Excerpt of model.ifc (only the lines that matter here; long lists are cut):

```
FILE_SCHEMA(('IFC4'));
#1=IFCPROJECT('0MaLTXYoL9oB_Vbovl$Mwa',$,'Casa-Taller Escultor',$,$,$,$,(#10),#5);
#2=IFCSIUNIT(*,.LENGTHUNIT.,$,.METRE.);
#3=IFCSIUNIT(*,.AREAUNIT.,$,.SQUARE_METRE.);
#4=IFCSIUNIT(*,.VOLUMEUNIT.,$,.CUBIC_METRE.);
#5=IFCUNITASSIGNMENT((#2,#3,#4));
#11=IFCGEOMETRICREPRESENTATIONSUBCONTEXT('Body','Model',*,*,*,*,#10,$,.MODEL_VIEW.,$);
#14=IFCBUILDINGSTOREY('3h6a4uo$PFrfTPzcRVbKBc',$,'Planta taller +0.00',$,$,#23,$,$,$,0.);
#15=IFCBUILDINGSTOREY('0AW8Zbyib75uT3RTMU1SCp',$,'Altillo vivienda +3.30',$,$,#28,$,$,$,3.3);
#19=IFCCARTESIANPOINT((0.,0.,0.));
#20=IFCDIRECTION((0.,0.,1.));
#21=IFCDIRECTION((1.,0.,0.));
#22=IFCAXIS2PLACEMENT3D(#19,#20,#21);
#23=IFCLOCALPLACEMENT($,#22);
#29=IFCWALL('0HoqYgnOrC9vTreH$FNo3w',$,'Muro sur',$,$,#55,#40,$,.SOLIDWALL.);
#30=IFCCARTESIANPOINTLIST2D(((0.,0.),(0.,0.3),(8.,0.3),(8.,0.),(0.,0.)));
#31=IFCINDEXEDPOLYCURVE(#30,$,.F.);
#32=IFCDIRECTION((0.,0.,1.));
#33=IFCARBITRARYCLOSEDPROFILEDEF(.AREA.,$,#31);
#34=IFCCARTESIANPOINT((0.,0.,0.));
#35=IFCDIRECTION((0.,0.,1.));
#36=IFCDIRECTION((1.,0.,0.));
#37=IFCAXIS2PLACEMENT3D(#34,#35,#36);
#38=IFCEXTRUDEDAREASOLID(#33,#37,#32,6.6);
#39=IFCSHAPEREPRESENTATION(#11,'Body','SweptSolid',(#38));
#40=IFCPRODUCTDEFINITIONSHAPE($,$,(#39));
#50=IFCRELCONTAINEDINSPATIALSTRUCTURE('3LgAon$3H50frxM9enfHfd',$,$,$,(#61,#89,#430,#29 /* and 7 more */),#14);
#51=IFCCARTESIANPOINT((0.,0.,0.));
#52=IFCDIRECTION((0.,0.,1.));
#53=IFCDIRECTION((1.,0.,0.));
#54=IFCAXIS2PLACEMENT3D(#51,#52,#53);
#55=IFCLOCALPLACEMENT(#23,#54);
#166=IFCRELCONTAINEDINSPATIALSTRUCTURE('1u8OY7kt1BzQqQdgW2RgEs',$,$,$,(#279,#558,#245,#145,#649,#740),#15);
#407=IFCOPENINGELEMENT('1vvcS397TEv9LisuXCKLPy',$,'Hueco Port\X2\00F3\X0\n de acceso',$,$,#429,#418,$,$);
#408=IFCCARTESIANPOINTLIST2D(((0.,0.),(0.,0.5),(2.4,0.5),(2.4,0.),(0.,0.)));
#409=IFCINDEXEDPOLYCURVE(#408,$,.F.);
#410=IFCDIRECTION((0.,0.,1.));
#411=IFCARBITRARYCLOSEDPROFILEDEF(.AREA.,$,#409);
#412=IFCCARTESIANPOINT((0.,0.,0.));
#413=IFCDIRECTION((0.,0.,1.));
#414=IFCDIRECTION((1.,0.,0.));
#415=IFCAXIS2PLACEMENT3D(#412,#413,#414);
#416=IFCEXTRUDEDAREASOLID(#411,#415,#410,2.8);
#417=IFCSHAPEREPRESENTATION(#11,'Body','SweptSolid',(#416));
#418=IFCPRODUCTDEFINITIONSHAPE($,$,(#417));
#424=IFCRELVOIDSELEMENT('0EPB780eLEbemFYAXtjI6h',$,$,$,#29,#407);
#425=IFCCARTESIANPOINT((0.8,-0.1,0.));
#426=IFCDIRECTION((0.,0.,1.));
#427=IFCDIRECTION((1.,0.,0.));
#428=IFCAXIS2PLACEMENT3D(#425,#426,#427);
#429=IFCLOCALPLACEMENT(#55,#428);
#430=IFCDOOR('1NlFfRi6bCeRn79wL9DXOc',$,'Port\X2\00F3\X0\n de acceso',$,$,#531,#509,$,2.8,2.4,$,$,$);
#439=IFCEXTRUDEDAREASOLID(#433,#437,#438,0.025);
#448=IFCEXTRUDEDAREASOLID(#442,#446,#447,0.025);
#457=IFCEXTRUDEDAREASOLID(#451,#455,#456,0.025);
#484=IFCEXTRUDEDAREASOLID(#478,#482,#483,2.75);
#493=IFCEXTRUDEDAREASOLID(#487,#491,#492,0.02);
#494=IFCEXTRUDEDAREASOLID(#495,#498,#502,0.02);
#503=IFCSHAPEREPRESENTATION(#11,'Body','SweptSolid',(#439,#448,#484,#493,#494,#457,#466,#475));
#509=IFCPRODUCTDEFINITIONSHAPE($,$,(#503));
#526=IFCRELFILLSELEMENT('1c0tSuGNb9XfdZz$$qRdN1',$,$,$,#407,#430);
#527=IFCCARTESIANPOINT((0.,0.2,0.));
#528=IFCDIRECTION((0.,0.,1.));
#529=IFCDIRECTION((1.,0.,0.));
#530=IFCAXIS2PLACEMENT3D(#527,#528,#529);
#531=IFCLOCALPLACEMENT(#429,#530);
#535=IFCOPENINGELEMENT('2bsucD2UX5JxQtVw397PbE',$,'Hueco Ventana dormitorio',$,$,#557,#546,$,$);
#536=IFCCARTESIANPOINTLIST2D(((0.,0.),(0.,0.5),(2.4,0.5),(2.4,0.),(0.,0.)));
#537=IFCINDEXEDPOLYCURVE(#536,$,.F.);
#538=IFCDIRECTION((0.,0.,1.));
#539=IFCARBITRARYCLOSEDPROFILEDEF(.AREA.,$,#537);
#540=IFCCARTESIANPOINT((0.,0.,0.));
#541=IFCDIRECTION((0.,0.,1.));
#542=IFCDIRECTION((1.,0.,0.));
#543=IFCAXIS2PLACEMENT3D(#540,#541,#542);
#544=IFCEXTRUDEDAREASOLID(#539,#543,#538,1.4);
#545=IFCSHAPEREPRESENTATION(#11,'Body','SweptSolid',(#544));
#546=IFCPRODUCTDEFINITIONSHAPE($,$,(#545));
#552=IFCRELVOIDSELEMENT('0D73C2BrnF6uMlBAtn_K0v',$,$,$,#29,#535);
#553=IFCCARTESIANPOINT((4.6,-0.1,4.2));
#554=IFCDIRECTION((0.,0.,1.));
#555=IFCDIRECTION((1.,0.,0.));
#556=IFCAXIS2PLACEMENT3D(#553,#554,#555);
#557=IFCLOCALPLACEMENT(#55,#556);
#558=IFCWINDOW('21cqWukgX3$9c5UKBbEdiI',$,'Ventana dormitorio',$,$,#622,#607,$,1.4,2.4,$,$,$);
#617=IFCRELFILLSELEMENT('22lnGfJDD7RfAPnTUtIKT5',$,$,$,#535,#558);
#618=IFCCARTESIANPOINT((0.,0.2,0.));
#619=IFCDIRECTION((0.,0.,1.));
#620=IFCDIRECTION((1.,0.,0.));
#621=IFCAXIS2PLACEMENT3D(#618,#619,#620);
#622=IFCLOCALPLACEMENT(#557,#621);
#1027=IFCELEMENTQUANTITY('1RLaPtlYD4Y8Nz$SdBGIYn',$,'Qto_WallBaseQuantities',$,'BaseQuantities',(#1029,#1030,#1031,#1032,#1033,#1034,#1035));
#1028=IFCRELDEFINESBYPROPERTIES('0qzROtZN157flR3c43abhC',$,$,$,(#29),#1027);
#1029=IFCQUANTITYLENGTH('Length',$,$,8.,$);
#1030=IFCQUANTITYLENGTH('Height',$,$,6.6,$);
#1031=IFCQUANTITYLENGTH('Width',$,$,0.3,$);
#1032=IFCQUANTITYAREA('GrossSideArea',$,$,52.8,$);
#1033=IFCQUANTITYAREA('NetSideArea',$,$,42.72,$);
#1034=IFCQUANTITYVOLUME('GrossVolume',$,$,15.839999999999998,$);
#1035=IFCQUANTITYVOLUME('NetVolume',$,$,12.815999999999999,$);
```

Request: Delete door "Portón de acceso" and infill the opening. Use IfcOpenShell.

```python
import ifcopenshell
import ifcopenshell.api.feature
import ifcopenshell.api.pset
import ifcopenshell.api.root
import ifcopenshell.geom
import ifcopenshell.util.element
import ifcopenshell.util.shape
import ifcopenshell.util.unit

model = ifcopenshell.open("model.ifc")
area_scale = ifcopenshell.util.unit.calculate_unit_scale(model, "AREAUNIT")
volume_scale = ifcopenshell.util.unit.calculate_unit_scale(model, "VOLUMEUNIT")
settings = ifcopenshell.geom.settings()


def volume(element):
    """Net volume in cubic metres, openings subtracted."""
    shape = ifcopenshell.geom.create_shape(settings, element)
    return ifcopenshell.util.shape.get_volume(shape.geometry)


door = model.by_id(430)
opening = door.FillsVoids[0].RelatingOpeningElement
wall = opening.VoidsElements[0].RelatingBuildingElement
before = volume(wall)

ifcopenshell.api.root.remove_product(model, product=door)
ifcopenshell.api.feature.remove_feature(model, feature=opening)

after = volume(wall)
thickness = 0.3  # wall thickness in metres

# Update the wall's stored quantities.
qto = model.by_id(ifcopenshell.util.element.get_pset(wall, "Qto_WallBaseQuantities", should_inherit=False)["id"])
ifcopenshell.api.pset.edit_qto(model, qto=qto, properties={
    "NetSideArea": after / thickness / area_scale,
    "NetVolume": after / volume_scale,
})

print(f"wall volume {before:.3f} -> {after:.3f} m3")

model.write("model_edited.ifc")
```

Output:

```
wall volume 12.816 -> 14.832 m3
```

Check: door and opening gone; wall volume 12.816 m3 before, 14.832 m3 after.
